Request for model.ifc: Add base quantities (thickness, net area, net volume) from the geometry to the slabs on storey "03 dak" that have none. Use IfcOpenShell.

First a look at what the model holds.

```python
import ifcopenshell
import ifcopenshell.util.element
import ifcopenshell.util.unit

model = ifcopenshell.open("model.ifc")
print(model.schema)
for unit_type in ("LENGTHUNIT", "AREAUNIT", "VOLUMEUNIT"):
    print(unit_type, ifcopenshell.util.unit.calculate_unit_scale(model, unit_type))
storey = next(s for s in model.by_type("IfcBuildingStorey") if s.Name == "03 dak")
slabs = [e for e in ifcopenshell.util.element.get_decomposition(storey) if e.is_a("IfcSlab")]
for e in sorted(slabs, key=lambda e: e.id()):
    print(e.id(), e.is_a(), e.Name, list(ifcopenshell.util.element.get_psets(e, qtos_only=True)), sep=" | ")
```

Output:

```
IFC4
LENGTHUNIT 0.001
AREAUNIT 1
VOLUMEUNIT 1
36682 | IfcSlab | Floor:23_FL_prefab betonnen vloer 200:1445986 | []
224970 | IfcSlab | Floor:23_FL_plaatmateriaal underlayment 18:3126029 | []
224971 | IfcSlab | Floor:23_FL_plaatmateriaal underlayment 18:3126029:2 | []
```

```python
import ifcopenshell
import ifcopenshell.api.pset
import ifcopenshell.geom
import ifcopenshell.util.element
import ifcopenshell.util.shape
import ifcopenshell.util.unit

model = ifcopenshell.open("model.ifc")
unit_scale = ifcopenshell.util.unit.calculate_unit_scale(model)
area_scale = ifcopenshell.util.unit.calculate_unit_scale(model, "AREAUNIT")
volume_scale = ifcopenshell.util.unit.calculate_unit_scale(model, "VOLUMEUNIT")
settings = ifcopenshell.geom.settings()

storey = next(s for s in model.by_type("IfcBuildingStorey") if s.Name == "03 dak")
slabs = [e for e in ifcopenshell.util.element.get_decomposition(storey) if e.is_a("IfcSlab")]

for e in sorted(slabs, key=lambda e: e.id()):
    if ifcopenshell.util.element.get_psets(e, qtos_only=True, should_inherit=False):
        continue
    # Geometry comes back in metres, in the element's own axes.
    shape = ifcopenshell.geom.create_shape(settings, e)
    values = {
        "Width": ifcopenshell.util.shape.get_z(shape.geometry) / unit_scale,
        "NetArea": ifcopenshell.util.shape.get_footprint_area(shape.geometry) / area_scale,
        "NetVolume": ifcopenshell.util.shape.get_volume(shape.geometry) / volume_scale,
    }
    qto = ifcopenshell.api.pset.add_qto(model, product=e, name="Qto_SlabBaseQuantities")
    ifcopenshell.api.pset.edit_qto(model, qto=qto, properties=values)
    print(e.id(), {k: round(v, 3) for k, v in values.items()})

model.write("model-out.ifc")
```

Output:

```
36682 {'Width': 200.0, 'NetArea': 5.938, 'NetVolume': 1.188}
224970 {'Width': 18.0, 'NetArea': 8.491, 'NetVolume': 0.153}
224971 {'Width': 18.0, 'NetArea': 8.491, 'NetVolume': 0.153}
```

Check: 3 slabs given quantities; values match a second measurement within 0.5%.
